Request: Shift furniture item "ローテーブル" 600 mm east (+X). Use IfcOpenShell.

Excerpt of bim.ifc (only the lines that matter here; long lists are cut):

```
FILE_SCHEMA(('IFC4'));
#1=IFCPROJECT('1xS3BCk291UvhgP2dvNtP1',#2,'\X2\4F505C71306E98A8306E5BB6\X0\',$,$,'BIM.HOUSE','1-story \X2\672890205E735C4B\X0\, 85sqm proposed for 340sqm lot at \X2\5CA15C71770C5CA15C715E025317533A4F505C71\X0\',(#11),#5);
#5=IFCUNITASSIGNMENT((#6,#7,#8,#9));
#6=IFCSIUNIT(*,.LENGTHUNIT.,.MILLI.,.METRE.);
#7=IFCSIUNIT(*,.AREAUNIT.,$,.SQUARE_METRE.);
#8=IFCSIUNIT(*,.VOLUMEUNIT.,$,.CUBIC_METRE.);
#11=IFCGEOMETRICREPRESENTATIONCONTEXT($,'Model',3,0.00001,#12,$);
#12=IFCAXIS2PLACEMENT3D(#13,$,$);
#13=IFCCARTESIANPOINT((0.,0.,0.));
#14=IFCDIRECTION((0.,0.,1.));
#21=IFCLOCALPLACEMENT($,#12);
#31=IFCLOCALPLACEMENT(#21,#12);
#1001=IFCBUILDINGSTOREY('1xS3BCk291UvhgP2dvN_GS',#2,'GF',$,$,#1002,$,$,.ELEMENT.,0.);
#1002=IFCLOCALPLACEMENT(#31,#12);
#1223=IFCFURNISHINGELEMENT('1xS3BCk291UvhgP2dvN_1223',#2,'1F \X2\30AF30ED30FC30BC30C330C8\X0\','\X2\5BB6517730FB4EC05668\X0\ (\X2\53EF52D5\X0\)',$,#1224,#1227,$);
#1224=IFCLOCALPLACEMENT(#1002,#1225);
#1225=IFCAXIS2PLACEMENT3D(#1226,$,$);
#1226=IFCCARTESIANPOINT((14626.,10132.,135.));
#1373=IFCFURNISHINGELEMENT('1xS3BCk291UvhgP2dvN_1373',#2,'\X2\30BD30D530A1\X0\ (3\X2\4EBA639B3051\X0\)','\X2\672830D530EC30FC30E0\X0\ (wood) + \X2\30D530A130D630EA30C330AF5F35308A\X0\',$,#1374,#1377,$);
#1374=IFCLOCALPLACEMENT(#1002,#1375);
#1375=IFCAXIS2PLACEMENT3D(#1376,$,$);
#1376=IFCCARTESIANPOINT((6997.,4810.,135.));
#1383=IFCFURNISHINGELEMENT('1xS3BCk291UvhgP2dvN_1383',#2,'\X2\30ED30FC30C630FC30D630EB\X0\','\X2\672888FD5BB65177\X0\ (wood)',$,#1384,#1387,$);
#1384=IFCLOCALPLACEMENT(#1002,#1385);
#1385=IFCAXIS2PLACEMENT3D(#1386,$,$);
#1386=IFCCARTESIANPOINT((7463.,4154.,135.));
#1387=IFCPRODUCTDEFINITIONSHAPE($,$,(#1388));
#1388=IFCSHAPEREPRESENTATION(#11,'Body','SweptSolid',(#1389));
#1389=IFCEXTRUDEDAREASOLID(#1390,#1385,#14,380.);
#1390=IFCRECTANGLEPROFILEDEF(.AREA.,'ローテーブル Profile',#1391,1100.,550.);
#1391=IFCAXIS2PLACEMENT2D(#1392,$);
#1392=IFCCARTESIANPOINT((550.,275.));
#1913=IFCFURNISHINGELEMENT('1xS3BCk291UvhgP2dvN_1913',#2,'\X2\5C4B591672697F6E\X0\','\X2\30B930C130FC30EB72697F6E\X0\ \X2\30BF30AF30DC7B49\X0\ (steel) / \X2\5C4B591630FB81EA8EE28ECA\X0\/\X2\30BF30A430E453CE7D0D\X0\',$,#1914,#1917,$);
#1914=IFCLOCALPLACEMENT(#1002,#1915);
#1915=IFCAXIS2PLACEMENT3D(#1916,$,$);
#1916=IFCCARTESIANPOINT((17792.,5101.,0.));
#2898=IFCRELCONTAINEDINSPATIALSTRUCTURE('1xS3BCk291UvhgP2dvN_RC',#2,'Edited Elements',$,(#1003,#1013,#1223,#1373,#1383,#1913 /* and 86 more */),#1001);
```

```python
import ifcopenshell
import ifcopenshell.api.geometry
import ifcopenshell.util.placement

model = ifcopenshell.open("bim.ifc")

item = model.by_id(1383)
matrix = ifcopenshell.util.placement.get_local_placement(item.ObjectPlacement)
matrix[0, 3] += 600.0
ifcopenshell.api.geometry.edit_object_placement(model, product=item, matrix=matrix, is_si=False)

print(ifcopenshell.util.placement.get_local_placement(item.ObjectPlacement).round(3) + 0.0)

model.write("bim_v2.ifc")
```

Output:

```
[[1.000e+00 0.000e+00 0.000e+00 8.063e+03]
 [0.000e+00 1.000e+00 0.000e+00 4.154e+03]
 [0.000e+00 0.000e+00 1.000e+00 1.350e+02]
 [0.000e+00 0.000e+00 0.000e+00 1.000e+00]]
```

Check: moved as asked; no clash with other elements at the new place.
